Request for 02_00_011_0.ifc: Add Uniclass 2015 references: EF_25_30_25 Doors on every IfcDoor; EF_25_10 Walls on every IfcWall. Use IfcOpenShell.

First a look at what the model holds.

```python
import ifcopenshell

model = ifcopenshell.open("02_00_011_0.ifc")
print(model.schema)
print("classifications:", [c.Name for c in model.by_type("IfcClassification")])
for ifc_class in ("IfcDoor", "IfcRoof", "IfcStair", "IfcWall", "IfcWindow"):
    print(ifc_class, len(model.by_type(ifc_class)))
```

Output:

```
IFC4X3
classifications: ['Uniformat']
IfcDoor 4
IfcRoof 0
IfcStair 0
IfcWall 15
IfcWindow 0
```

```python
import ifcopenshell
import ifcopenshell.api.classification

model = ifcopenshell.open("02_00_011_0.ifc")

system = ifcopenshell.api.classification.add_classification(model, classification="Uniclass 2015")

codes = {
    "IfcDoor": ("EF_25_30_25", "Doors"),
    "IfcWall": ("EF_25_10", "Walls"),
}
for ifc_class, (code, name) in codes.items():
    products = model.by_type(ifc_class)
    ifcopenshell.api.classification.add_reference(
        model, products=products, classification=system, identification=code, name=name
    )
    print(code, len(products))

model.write("02_00_011_0_edited.ifc")
```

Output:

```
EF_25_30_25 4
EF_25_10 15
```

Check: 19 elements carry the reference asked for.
